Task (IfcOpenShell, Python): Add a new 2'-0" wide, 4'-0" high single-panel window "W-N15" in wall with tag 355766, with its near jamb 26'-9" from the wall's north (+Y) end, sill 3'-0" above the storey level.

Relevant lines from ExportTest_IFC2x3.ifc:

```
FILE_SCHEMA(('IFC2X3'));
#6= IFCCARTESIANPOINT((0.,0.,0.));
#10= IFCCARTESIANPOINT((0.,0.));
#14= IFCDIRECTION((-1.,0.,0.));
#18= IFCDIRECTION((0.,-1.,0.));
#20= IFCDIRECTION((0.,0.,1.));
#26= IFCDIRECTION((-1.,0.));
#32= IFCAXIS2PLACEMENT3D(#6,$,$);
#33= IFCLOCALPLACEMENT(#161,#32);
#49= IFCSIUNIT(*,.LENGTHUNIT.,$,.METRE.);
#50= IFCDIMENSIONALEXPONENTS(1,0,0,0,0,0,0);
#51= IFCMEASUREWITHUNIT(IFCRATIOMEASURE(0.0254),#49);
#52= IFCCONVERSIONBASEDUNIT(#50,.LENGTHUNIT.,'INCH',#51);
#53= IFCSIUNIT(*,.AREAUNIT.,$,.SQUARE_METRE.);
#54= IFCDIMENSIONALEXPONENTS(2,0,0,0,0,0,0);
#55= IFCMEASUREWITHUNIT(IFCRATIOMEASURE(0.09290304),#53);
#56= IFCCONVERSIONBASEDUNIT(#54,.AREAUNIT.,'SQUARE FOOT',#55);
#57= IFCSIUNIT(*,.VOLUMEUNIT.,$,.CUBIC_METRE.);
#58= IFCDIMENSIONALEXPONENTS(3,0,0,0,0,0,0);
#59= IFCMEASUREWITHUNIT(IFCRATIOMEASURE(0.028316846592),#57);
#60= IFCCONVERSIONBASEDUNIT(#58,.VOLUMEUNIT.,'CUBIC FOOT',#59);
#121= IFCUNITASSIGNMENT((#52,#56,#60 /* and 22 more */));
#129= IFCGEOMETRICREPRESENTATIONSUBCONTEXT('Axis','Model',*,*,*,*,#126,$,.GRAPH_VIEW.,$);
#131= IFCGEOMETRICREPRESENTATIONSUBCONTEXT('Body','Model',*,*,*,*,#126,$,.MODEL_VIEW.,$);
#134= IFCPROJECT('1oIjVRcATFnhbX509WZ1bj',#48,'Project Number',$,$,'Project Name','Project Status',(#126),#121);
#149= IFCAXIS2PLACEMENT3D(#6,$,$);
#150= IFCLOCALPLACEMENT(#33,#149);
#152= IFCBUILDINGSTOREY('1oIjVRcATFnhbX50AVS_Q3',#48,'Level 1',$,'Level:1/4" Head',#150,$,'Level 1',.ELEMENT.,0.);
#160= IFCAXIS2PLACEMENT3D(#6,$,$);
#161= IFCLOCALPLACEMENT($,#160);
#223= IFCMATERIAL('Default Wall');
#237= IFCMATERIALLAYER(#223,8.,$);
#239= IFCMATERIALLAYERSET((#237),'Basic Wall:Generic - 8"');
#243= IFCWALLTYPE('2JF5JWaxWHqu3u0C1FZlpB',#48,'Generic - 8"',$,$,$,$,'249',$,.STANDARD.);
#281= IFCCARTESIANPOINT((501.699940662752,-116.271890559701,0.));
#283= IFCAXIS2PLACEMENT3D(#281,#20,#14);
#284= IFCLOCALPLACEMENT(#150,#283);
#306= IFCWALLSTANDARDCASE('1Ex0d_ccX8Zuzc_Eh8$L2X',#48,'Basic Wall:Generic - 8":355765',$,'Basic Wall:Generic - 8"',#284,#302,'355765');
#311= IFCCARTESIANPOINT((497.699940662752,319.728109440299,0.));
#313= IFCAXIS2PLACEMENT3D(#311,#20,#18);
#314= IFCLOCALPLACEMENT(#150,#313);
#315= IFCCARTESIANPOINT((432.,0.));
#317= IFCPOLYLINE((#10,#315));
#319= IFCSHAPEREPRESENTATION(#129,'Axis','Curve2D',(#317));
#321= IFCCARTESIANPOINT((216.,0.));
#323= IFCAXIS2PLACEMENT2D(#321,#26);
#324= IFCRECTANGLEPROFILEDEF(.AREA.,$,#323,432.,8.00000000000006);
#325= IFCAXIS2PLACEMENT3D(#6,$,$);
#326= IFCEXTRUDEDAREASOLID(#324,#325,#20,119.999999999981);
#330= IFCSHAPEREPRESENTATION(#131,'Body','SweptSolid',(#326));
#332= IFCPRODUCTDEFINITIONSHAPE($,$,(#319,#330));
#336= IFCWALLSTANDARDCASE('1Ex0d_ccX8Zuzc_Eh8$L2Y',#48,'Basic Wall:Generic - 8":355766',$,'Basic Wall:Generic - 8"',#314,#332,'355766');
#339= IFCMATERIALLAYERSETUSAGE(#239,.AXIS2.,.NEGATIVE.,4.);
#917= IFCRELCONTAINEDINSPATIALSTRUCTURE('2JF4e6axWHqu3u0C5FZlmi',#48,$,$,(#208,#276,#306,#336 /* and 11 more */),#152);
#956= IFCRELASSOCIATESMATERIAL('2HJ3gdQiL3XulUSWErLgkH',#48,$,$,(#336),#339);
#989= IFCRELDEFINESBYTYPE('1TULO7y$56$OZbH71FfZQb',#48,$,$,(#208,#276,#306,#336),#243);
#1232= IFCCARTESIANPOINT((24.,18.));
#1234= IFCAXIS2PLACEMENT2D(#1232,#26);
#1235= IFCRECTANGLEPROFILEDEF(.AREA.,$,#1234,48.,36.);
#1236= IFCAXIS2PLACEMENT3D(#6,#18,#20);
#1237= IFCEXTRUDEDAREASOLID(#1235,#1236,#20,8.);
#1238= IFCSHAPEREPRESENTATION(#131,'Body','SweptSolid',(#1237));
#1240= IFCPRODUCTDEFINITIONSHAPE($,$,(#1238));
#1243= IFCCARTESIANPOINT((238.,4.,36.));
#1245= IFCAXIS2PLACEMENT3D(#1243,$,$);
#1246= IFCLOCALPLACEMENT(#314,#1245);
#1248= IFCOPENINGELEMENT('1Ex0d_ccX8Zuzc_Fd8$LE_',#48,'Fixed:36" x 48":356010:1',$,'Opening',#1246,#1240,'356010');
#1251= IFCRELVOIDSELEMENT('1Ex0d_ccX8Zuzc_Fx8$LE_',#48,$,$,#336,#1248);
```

```python
import numpy as np
import ifcopenshell
import ifcopenshell.api.feature
import ifcopenshell.api.geometry
import ifcopenshell.api.root
import ifcopenshell.api.spatial
import ifcopenshell.api.type
import ifcopenshell.geom
import ifcopenshell.util.element
import ifcopenshell.util.placement
import ifcopenshell.util.representation
import ifcopenshell.util.shape
import ifcopenshell.util.unit

model = ifcopenshell.open("ExportTest_IFC2x3.ifc")
unit_scale = ifcopenshell.util.unit.calculate_unit_scale(model)
settings = ifcopenshell.geom.settings()


def volume(element):
    """Net volume in cubic metres, openings subtracted."""
    shape = ifcopenshell.geom.create_shape(settings, element)
    return ifcopenshell.util.shape.get_volume(shape.geometry)


wall = model.by_id(336)
storey = ifcopenshell.util.element.get_container(wall, ifc_class="IfcBuildingStorey")
context = ifcopenshell.util.representation.get_context(model, "Model", "Body", "MODEL_VIEW")
before = volume(wall)

width, height, from_end, sill = 0.6096, 1.2192, 8.1534, 0.9144  # metres

# The wall runs along its own X axis, and the end named is its -X end.
wall_shape = ifcopenshell.geom.create_shape(settings, wall)
x, y, z = ifcopenshell.util.shape.get_vertices(wall_shape.geometry).T
start = x.min() + from_end
face, thickness = float(y.min()), float(y.max() - y.min())
wall_matrix = ifcopenshell.util.placement.get_local_placement(wall.ObjectPlacement)
level = ifcopenshell.util.placement.get_local_placement(storey.ObjectPlacement)[2, 3]


def in_wall(x, y):
    """Placement at x, y metres in the wall's axes, at sill height."""
    matrix = wall_matrix.copy()
    matrix[:, 3] = wall_matrix @ np.array([x / unit_scale, y / unit_scale, 0.0, 1.0])
    matrix[2, 3] = level + sill / unit_scale
    return matrix


# Opening: a box that overshoots both wall faces by 50 mm.
opening = ifcopenshell.api.root.create_entity(model, ifc_class="IfcOpeningElement")
box = ifcopenshell.api.geometry.add_wall_representation(
    model, context=context, length=width, height=height, thickness=thickness + 0.1
)
ifcopenshell.api.geometry.assign_representation(model, product=opening, representation=box)
ifcopenshell.api.geometry.edit_object_placement(model, product=opening, matrix=in_wall(start, face - 0.05), is_si=False)
ifcopenshell.api.feature.add_feature(model, feature=opening, element=wall)

window = ifcopenshell.api.root.create_entity(model, ifc_class="IfcWindow", name="W-N15")
window.OverallWidth, window.OverallHeight = width / unit_scale, height / unit_scale
body = ifcopenshell.api.geometry.add_window_representation(
    model,
    context=context,
    overall_width=window.OverallWidth,
    overall_height=window.OverallHeight,
    partition_type="SINGLE_PANEL",
)
ifcopenshell.api.geometry.assign_representation(model, product=window, representation=body)
ifcopenshell.api.spatial.assign_container(model, products=[window], relating_structure=storey)
fills = ifcopenshell.api.feature.add_filling(model, opening=opening, element=window)
fills.OwnerHistory = window.OwnerHistory  # required in IFC2X3

# IFC2X3 keeps the operation on the window style.
style = ifcopenshell.api.root.create_entity(model, ifc_class="IfcWindowStyle", name="W-N15")
style.OperationType, style.ConstructionType = "SINGLE_PANEL", "NOTDEFINED"
style.ParameterTakesPrecedence = style.Sizeable = False
ifcopenshell.api.type.assign_type(model, related_objects=[window], relating_type=style)

# Centre the window in the wall's thickness.
ifcopenshell.api.geometry.edit_object_placement(model, product=window, matrix=in_wall(start, face), is_si=False)
window_shape = ifcopenshell.geom.create_shape(settings, window)
depth = ifcopenshell.util.shape.get_vertices(window_shape.geometry)[:, 1]
offset = face + thickness / 2 - (depth.min() + depth.max()) / 2
ifcopenshell.api.geometry.edit_object_placement(model, product=window, matrix=in_wall(start, offset), is_si=False)

after = volume(wall)

print(f"wall volume {before:.3f} -> {after:.3f} m3")

model.write("ExportTest_IFC2x3_rev.ifc")
```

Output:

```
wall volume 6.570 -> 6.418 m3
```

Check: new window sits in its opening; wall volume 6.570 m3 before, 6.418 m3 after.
